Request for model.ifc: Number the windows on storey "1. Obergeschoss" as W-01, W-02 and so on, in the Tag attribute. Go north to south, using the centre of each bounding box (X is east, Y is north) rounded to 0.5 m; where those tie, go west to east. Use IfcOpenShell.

First a look at what the model holds.

```python
import ifcopenshell
import ifcopenshell.util.element
import ifcopenshell.util.placement

model = ifcopenshell.open("model.ifc")
print(model.schema)
storey = next(s for s in model.by_type("IfcBuildingStorey") if s.Name == "1. Obergeschoss")
windows = [e for e in ifcopenshell.util.element.get_decomposition(storey) if e.is_a("IfcWindow")]
for e in sorted(windows, key=lambda e: e.id()):
    origin = ifcopenshell.util.placement.get_local_placement(e.ObjectPlacement)[:3, 3]
    print(e.id(), e.Tag, e.Name, origin.round(2) + 0.0, sep=" | ")
```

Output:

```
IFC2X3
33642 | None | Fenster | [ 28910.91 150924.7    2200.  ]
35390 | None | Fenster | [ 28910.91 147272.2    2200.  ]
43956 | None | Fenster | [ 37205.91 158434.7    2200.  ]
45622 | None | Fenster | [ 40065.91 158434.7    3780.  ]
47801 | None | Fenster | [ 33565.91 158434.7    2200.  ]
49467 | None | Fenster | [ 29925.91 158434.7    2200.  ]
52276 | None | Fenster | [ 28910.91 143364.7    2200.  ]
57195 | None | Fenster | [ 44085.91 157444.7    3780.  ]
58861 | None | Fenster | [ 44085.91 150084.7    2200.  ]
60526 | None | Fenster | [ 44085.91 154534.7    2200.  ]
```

```python
import ifcopenshell
import ifcopenshell.geom
import ifcopenshell.util.element
import ifcopenshell.util.shape

model = ifcopenshell.open("model.ifc")
settings = ifcopenshell.geom.settings()
settings.set("use-world-coords", True)


def centre(element):
    shape = ifcopenshell.geom.create_shape(settings, element)
    return ifcopenshell.util.shape.get_bbox_centroid(shape.geometry)


storey = next(s for s in model.by_type("IfcBuildingStorey") if s.Name == "1. Obergeschoss")
windows = [e for e in ifcopenshell.util.element.get_decomposition(storey) if e.is_a("IfcWindow")]

# Insertion points can sit at a corner or the storey origin, so sort by the geometry (in metres).
centres = {e: centre(e) for e in windows}
windows.sort(key=lambda e: (-round(centres[e][1] / 0.5), centres[e][0]))

for i, e in enumerate(windows, start=1):
    number = f"W-{i:02d}"
    e.Tag = number
    print(e.id(), number)

model.write("model_edited.ifc")
```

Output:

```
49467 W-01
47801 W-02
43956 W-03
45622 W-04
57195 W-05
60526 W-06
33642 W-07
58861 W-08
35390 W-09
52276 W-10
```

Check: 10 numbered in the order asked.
